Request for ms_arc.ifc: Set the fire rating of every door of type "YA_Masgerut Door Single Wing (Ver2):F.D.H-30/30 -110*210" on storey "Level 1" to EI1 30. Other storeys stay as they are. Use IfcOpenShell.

First a look at what the model holds.

```python
import ifcopenshell
import ifcopenshell.util.element

model = ifcopenshell.open("ms_arc.ifc")
print(model.schema)
storey = next(s for s in model.by_type("IfcBuildingStorey") if s.Name == "Level 1")
doors = [e for e in ifcopenshell.util.element.get_decomposition(storey) if e.is_a("IfcDoor")]
seen = {}
for e in doors:
    element_type = ifcopenshell.util.element.get_type(e)
    key = (element_type.Name if element_type != e and element_type else None, ifcopenshell.util.element.get_pset(e, "Pset_DoorCommon", "FireRating"))
    seen[key] = seen.get(key, 0) + 1
for (name, value), count in sorted(seen.items(), key=str):
    print(count, "x", name, "|", value)
```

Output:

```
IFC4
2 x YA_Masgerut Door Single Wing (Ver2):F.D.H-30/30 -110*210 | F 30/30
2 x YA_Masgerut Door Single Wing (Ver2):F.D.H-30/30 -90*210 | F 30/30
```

```python
import ifcopenshell
import ifcopenshell.api.pset
import ifcopenshell.util.element

model = ifcopenshell.open("ms_arc.ifc")

storey = next(s for s in model.by_type("IfcBuildingStorey") if s.Name == "Level 1")
doors = [e for e in ifcopenshell.util.element.get_decomposition(storey) if e.is_a("IfcDoor")]

count = 0
for e in doors:
    element_type = ifcopenshell.util.element.get_type(e)
    if element_type in (None, e) or element_type.Name != "YA_Masgerut Door Single Wing (Ver2):F.D.H-30/30 -110*210":
        continue
    # add_pset returns the element's existing set when there is one.
    pset = ifcopenshell.api.pset.add_pset(model, product=e, name="Pset_DoorCommon")
    ifcopenshell.api.pset.edit_pset(model, pset=pset, properties={"FireRating": "EI1 30"})
    count += 1

print(count, "doors updated")

model.write("ms_arc_edited.ifc")
```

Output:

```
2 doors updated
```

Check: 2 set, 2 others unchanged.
